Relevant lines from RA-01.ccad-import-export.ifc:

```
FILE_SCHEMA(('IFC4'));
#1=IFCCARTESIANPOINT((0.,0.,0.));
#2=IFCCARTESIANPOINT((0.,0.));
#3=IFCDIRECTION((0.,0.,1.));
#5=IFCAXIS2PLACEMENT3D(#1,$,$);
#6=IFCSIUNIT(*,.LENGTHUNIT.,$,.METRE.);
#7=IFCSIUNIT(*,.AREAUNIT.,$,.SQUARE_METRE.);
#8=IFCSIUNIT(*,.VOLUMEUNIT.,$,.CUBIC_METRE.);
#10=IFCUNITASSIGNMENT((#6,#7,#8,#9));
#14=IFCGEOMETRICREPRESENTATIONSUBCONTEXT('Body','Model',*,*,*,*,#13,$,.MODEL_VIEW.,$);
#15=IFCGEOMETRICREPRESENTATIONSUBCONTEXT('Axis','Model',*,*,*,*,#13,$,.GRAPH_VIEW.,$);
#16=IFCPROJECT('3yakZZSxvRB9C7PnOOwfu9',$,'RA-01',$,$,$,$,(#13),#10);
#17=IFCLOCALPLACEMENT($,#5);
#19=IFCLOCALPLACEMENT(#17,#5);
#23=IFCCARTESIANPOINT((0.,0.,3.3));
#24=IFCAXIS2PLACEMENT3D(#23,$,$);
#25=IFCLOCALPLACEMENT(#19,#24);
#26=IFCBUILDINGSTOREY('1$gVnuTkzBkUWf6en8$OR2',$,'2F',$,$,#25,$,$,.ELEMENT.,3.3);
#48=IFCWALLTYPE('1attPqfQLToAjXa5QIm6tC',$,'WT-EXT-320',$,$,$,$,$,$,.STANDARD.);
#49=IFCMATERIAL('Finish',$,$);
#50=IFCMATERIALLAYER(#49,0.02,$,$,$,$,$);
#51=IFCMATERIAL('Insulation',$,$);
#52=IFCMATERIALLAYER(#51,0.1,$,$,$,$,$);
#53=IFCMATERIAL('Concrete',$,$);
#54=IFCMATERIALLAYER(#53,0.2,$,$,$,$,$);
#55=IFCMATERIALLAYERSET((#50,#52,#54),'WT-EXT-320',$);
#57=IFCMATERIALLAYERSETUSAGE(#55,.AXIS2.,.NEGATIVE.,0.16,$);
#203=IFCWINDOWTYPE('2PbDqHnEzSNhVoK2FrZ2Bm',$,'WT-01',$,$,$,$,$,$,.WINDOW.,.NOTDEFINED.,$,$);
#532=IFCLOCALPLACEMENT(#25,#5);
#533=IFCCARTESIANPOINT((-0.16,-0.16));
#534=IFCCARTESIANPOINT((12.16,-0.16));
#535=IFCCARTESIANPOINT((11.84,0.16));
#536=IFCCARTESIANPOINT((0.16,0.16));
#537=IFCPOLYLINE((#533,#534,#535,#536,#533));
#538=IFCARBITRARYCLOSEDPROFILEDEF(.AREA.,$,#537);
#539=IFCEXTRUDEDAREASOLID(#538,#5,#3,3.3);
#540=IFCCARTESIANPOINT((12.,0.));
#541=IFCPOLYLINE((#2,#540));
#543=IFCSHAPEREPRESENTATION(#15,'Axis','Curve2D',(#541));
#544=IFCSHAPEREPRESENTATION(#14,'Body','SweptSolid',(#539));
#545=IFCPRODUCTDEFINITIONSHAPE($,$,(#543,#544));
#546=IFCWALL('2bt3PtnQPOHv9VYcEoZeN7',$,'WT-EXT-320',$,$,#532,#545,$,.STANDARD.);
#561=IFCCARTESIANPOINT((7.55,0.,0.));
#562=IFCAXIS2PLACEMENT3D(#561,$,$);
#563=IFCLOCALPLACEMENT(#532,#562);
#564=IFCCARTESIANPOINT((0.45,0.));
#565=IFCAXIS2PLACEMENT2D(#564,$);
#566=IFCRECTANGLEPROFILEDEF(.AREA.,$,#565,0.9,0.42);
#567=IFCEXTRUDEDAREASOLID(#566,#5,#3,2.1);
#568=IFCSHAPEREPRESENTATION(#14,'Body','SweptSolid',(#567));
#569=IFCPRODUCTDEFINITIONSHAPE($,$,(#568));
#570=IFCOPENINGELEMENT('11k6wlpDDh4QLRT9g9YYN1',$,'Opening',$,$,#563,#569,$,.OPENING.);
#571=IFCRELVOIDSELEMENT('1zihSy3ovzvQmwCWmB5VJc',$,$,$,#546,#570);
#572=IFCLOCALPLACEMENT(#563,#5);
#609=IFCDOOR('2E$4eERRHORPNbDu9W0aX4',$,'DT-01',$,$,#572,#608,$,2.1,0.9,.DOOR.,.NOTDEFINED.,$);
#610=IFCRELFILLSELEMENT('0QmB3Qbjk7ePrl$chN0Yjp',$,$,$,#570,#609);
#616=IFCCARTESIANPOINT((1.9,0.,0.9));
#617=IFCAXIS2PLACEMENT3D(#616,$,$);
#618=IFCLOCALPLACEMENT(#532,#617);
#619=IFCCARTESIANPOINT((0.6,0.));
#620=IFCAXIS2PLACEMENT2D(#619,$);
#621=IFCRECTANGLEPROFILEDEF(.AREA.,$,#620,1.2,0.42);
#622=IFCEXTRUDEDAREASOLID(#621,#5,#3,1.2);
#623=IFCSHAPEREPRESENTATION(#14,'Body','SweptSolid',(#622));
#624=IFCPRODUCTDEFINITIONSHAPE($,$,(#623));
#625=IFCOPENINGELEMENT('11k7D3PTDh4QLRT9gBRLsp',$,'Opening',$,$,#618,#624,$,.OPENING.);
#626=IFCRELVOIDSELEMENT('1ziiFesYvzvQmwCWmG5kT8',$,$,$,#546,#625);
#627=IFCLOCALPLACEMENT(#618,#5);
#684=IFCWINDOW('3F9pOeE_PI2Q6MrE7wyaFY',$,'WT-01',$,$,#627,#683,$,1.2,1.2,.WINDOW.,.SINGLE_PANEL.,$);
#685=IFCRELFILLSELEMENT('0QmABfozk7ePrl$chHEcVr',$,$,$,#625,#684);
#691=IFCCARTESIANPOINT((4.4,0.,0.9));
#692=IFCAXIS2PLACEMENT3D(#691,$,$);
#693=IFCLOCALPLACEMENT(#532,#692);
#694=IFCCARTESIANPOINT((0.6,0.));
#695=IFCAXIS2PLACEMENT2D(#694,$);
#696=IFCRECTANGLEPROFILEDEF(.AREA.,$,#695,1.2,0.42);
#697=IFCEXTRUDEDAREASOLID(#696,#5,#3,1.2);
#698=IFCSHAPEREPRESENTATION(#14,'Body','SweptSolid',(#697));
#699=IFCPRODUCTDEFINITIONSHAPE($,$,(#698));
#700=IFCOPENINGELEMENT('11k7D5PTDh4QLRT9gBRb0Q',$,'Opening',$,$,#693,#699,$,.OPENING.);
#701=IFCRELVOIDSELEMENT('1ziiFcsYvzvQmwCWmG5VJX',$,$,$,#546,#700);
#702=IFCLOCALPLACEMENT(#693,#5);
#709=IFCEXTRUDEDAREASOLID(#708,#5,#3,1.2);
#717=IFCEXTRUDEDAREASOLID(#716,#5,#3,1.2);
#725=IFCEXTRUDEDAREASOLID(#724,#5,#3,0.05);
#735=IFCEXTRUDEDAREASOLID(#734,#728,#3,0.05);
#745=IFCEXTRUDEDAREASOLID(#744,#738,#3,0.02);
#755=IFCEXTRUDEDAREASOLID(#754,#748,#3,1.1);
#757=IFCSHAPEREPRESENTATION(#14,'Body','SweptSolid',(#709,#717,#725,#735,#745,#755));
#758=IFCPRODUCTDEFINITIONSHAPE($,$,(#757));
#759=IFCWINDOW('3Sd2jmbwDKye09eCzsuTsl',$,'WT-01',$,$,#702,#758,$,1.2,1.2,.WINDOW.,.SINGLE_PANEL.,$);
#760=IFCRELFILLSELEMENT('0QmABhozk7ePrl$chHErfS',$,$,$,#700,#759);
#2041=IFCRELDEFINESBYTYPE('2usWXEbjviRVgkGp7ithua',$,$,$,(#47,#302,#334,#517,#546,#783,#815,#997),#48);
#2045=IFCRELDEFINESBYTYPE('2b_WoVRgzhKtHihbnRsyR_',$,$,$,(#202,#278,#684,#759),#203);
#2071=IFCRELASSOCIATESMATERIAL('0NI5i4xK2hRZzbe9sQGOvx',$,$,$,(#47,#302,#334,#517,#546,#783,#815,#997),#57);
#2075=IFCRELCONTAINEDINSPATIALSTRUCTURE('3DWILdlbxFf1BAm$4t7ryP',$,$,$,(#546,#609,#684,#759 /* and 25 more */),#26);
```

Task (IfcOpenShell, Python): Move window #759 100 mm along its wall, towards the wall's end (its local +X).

```python
import ifcopenshell
import ifcopenshell.api.geometry
import ifcopenshell.util.placement
import ifcopenshell.util.unit

model = ifcopenshell.open("RA-01.ccad-import-export.ifc")
unit_scale = ifcopenshell.util.unit.calculate_unit_scale(model)

window = model.by_guid("3Sd2jmbwDKye09eCzsuTsl")
opening = window.FillsVoids[0].RelatingOpeningElement
wall = opening.VoidsElements[0].RelatingBuildingElement

wall_matrix = ifcopenshell.util.placement.get_local_placement(wall.ObjectPlacement)
shift = wall_matrix[:3, 0] * 0.1 / unit_scale
before = ifcopenshell.util.placement.get_local_placement(window.ObjectPlacement)[:3, 3].copy()

# The window is placed relative to its opening, so it follows when the opening moves.
matrix = ifcopenshell.util.placement.get_local_placement(opening.ObjectPlacement)
matrix[:3, 3] += shift
ifcopenshell.api.geometry.edit_object_placement(
    model, product=opening, matrix=matrix, is_si=False, should_transform_children=True
)

after = ifcopenshell.util.placement.get_local_placement(window.ObjectPlacement)[:3, 3]
print("window moved by", (after - before).round(3) + 0.0)

model.write("RA-01.ccad-import-export_rev.ifc")
```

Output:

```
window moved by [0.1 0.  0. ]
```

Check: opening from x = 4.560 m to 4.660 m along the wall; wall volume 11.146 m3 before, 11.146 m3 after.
